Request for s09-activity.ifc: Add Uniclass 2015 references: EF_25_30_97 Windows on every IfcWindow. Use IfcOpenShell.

First a look at what the model holds.

```python
import ifcopenshell

model = ifcopenshell.open("s09-activity.ifc")
print(model.schema)
print("classifications:", [c.Name for c in model.by_type("IfcClassification")])
for ifc_class in ("IfcDoor", "IfcRoof", "IfcStair", "IfcWall", "IfcWindow"):
    print(ifc_class, len(model.by_type(ifc_class)))
```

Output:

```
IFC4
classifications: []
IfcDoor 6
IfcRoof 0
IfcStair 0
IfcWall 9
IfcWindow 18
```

```python
import ifcopenshell
import ifcopenshell.api.classification

model = ifcopenshell.open("s09-activity.ifc")

system = ifcopenshell.api.classification.add_classification(model, classification="Uniclass 2015")

codes = {
    "IfcWindow": ("EF_25_30_97", "Windows"),
}
for ifc_class, (code, name) in codes.items():
    products = model.by_type(ifc_class)
    ifcopenshell.api.classification.add_reference(
        model, products=products, classification=system, identification=code, name=name
    )
    print(code, len(products))

model.write("s09-activity-out.ifc")
```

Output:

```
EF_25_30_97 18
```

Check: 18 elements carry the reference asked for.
